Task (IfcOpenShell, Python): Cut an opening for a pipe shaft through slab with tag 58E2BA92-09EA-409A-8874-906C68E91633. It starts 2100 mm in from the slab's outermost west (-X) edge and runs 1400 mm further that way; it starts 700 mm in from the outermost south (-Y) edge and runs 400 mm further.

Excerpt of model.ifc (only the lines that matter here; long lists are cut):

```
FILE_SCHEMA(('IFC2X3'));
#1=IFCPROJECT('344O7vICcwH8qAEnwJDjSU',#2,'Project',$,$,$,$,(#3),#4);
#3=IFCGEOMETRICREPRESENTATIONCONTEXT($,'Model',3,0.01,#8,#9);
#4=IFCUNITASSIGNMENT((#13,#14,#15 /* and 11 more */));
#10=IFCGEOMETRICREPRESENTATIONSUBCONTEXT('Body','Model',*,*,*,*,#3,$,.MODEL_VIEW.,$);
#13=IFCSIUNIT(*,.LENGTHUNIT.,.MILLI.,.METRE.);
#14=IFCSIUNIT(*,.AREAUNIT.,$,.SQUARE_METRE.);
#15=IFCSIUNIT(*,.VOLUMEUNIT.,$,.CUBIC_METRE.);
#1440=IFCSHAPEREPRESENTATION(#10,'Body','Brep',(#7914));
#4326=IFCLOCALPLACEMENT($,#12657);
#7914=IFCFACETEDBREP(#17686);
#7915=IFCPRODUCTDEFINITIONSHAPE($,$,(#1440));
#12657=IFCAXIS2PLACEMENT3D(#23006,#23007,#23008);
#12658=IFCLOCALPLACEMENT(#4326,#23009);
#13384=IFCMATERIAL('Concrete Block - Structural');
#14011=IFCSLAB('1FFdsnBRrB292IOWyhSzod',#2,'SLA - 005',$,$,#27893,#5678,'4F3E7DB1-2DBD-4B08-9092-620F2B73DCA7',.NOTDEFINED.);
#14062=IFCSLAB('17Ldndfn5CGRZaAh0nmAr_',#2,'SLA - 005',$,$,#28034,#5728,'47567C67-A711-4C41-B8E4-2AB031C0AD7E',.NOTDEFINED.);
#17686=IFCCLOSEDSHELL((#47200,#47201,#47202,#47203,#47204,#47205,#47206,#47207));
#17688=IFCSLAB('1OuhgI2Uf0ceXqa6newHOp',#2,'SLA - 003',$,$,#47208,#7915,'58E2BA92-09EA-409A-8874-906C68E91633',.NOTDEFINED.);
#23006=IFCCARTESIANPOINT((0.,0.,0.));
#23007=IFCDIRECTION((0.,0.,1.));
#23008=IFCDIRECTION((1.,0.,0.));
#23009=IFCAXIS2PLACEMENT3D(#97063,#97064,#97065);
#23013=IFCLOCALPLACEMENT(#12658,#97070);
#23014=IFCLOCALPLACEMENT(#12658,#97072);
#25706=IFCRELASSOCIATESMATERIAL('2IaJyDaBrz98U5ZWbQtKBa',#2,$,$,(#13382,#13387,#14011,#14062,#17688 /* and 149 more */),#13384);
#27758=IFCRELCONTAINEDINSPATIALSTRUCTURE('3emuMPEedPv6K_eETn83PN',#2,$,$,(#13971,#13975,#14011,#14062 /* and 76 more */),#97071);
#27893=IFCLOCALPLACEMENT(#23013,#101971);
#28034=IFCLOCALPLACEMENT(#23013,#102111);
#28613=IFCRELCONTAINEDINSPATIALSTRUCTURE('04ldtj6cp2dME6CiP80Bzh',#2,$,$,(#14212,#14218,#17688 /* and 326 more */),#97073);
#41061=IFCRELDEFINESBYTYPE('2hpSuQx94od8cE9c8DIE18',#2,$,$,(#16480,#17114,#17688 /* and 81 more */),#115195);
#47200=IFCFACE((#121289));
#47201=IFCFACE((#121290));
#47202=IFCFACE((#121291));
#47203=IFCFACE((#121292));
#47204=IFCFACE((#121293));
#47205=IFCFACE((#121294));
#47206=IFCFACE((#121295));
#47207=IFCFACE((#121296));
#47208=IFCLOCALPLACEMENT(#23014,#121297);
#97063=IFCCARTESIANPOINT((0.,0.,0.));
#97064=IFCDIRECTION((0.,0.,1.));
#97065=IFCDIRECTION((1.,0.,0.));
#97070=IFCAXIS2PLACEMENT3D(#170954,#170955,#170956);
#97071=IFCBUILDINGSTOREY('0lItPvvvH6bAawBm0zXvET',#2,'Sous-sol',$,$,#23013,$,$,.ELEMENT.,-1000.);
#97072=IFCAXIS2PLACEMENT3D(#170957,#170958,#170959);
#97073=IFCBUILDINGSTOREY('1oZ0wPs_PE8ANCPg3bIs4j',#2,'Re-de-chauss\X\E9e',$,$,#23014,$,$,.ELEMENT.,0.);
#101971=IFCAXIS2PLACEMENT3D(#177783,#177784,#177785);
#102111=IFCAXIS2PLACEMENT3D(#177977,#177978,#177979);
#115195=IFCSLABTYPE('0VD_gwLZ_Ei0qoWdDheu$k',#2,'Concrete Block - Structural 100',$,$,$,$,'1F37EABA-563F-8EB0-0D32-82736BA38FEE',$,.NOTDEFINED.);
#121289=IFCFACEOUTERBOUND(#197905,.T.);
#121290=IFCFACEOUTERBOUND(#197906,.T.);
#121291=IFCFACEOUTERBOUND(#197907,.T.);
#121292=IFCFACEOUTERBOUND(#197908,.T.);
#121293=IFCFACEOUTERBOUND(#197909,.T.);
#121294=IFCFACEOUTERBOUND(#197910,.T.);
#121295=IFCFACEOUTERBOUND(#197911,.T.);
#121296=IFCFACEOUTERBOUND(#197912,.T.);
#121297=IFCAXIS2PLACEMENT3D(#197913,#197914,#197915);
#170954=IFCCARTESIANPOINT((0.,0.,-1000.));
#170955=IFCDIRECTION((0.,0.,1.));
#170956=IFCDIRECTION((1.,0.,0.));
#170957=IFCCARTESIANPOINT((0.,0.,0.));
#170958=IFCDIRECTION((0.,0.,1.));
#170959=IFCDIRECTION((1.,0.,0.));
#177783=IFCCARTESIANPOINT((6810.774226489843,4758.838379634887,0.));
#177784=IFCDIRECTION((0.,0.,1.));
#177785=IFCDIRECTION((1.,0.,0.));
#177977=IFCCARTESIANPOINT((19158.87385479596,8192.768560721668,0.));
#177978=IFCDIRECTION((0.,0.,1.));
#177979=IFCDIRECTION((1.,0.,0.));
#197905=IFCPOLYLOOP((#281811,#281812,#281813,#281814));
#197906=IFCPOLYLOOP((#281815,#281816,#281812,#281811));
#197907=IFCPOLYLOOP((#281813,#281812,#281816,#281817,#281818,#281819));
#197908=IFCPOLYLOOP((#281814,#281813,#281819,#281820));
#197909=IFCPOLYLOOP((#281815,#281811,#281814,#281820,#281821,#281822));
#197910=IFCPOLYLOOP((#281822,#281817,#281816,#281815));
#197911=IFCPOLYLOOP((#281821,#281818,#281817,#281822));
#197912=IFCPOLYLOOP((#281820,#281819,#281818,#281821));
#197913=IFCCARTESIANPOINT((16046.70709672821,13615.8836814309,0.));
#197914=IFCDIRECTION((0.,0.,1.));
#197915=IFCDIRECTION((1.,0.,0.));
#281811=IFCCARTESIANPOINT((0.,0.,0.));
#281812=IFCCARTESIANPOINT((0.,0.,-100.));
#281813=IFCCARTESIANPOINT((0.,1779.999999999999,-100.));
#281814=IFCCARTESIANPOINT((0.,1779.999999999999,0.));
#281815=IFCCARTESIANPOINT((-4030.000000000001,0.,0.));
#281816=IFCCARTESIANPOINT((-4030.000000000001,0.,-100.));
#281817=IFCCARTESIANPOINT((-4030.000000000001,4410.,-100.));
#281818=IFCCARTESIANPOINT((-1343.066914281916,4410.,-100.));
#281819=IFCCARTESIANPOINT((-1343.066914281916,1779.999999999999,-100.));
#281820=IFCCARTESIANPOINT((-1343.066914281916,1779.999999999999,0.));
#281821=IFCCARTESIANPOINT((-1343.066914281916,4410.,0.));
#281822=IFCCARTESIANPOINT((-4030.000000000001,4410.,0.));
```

```python
import numpy as np
import ifcopenshell
import ifcopenshell.api.feature
import ifcopenshell.api.geometry
import ifcopenshell.api.root
import ifcopenshell.geom
import ifcopenshell.util.placement
import ifcopenshell.util.representation
import ifcopenshell.util.shape
import ifcopenshell.util.unit

model = ifcopenshell.open("model.ifc")
unit_scale = ifcopenshell.util.unit.calculate_unit_scale(model)
settings = ifcopenshell.geom.settings()


def volume(element):
    """Net volume in cubic metres, openings subtracted."""
    shape = ifcopenshell.geom.create_shape(settings, element)
    return ifcopenshell.util.shape.get_volume(shape.geometry)


slab = model.by_id(17688)
before = volume(slab)

# Extent in the slab's own axes, in metres. The edges named are its -X and -Y sides.
slab_shape = ifcopenshell.geom.create_shape(settings, slab)
vertices = ifcopenshell.util.shape.get_vertices(slab_shape.geometry)
x_min, y_min, bottom = vertices.min(axis=0)
top = vertices[:, 2].max()

opening = ifcopenshell.api.root.create_entity(model, ifc_class="IfcOpeningElement", name="Pipe shaft opening")
context = ifcopenshell.util.representation.get_context(model, "Model", "Body", "MODEL_VIEW")
width, depth = 1.4, 0.4
outline = [(0.0, 0.0), (width, 0.0), (width, depth), (0.0, depth), (0.0, 0.0)]
# Overshoot both faces by 50 mm so the cut is clean.
shape = ifcopenshell.api.geometry.add_slab_representation(
    model, context=context, depth=top - bottom + 0.1, polyline=outline
)
ifcopenshell.api.geometry.assign_representation(model, product=opening, representation=shape)

matrix = ifcopenshell.util.placement.get_local_placement(slab.ObjectPlacement)
matrix[:, 3] = matrix @ np.append(np.array([x_min + 2.1, y_min + 0.7, bottom - 0.05]) / unit_scale, 1.0)
ifcopenshell.api.geometry.edit_object_placement(model, product=opening, matrix=matrix, is_si=False)
ifcopenshell.api.feature.add_feature(model, feature=opening, element=slab)

after = volume(slab)

print(f"slab volume {before:.3f} -> {after:.3f} m3")

model.write("model_rev.ifc")
```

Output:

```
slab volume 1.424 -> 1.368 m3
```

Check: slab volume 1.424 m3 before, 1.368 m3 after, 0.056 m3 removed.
